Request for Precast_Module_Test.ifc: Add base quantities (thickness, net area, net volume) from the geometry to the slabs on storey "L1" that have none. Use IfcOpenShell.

First a look at what the model holds.

```python
import ifcopenshell
import ifcopenshell.util.element
import ifcopenshell.util.unit

model = ifcopenshell.open("Precast_Module_Test.ifc")
print(model.schema)
for unit_type in ("LENGTHUNIT", "AREAUNIT", "VOLUMEUNIT"):
    print(unit_type, ifcopenshell.util.unit.calculate_unit_scale(model, unit_type))
storey = next(s for s in model.by_type("IfcBuildingStorey") if s.Name == "L1")
slabs = [e for e in ifcopenshell.util.element.get_decomposition(storey) if e.is_a("IfcSlab")]
for e in sorted(slabs, key=lambda e: e.id()):
    print(e.id(), e.is_a(), e.Name, list(ifcopenshell.util.element.get_psets(e, qtos_only=True)), sep=" | ")
```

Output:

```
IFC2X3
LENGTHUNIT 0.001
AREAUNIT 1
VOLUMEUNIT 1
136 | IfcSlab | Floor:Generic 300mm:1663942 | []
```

```python
import ifcopenshell
import ifcopenshell.api.pset
import ifcopenshell.geom
import ifcopenshell.util.element
import ifcopenshell.util.shape
import ifcopenshell.util.unit

model = ifcopenshell.open("Precast_Module_Test.ifc")
unit_scale = ifcopenshell.util.unit.calculate_unit_scale(model)
area_scale = ifcopenshell.util.unit.calculate_unit_scale(model, "AREAUNIT")
volume_scale = ifcopenshell.util.unit.calculate_unit_scale(model, "VOLUMEUNIT")
settings = ifcopenshell.geom.settings()

storey = next(s for s in model.by_type("IfcBuildingStorey") if s.Name == "L1")
slabs = [e for e in ifcopenshell.util.element.get_decomposition(storey) if e.is_a("IfcSlab")]

for e in sorted(slabs, key=lambda e: e.id()):
    if ifcopenshell.util.element.get_psets(e, qtos_only=True, should_inherit=False):
        continue
    # Geometry comes back in metres, in the element's own axes.
    shape = ifcopenshell.geom.create_shape(settings, e)
    values = {
        "Width": ifcopenshell.util.shape.get_z(shape.geometry) / unit_scale,
        "NetArea": ifcopenshell.util.shape.get_footprint_area(shape.geometry) / area_scale,
        "NetVolume": ifcopenshell.util.shape.get_volume(shape.geometry) / volume_scale,
    }
    qto = ifcopenshell.api.pset.add_qto(model, product=e, name="BaseQuantities")
    ifcopenshell.api.pset.edit_qto(model, qto=qto, properties=values)
    print(e.id(), {k: round(v, 3) for k, v in values.items()})

model.write("Precast_Module_Test_rev.ifc")
```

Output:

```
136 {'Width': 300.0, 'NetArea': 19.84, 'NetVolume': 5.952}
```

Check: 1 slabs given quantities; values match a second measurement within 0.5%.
